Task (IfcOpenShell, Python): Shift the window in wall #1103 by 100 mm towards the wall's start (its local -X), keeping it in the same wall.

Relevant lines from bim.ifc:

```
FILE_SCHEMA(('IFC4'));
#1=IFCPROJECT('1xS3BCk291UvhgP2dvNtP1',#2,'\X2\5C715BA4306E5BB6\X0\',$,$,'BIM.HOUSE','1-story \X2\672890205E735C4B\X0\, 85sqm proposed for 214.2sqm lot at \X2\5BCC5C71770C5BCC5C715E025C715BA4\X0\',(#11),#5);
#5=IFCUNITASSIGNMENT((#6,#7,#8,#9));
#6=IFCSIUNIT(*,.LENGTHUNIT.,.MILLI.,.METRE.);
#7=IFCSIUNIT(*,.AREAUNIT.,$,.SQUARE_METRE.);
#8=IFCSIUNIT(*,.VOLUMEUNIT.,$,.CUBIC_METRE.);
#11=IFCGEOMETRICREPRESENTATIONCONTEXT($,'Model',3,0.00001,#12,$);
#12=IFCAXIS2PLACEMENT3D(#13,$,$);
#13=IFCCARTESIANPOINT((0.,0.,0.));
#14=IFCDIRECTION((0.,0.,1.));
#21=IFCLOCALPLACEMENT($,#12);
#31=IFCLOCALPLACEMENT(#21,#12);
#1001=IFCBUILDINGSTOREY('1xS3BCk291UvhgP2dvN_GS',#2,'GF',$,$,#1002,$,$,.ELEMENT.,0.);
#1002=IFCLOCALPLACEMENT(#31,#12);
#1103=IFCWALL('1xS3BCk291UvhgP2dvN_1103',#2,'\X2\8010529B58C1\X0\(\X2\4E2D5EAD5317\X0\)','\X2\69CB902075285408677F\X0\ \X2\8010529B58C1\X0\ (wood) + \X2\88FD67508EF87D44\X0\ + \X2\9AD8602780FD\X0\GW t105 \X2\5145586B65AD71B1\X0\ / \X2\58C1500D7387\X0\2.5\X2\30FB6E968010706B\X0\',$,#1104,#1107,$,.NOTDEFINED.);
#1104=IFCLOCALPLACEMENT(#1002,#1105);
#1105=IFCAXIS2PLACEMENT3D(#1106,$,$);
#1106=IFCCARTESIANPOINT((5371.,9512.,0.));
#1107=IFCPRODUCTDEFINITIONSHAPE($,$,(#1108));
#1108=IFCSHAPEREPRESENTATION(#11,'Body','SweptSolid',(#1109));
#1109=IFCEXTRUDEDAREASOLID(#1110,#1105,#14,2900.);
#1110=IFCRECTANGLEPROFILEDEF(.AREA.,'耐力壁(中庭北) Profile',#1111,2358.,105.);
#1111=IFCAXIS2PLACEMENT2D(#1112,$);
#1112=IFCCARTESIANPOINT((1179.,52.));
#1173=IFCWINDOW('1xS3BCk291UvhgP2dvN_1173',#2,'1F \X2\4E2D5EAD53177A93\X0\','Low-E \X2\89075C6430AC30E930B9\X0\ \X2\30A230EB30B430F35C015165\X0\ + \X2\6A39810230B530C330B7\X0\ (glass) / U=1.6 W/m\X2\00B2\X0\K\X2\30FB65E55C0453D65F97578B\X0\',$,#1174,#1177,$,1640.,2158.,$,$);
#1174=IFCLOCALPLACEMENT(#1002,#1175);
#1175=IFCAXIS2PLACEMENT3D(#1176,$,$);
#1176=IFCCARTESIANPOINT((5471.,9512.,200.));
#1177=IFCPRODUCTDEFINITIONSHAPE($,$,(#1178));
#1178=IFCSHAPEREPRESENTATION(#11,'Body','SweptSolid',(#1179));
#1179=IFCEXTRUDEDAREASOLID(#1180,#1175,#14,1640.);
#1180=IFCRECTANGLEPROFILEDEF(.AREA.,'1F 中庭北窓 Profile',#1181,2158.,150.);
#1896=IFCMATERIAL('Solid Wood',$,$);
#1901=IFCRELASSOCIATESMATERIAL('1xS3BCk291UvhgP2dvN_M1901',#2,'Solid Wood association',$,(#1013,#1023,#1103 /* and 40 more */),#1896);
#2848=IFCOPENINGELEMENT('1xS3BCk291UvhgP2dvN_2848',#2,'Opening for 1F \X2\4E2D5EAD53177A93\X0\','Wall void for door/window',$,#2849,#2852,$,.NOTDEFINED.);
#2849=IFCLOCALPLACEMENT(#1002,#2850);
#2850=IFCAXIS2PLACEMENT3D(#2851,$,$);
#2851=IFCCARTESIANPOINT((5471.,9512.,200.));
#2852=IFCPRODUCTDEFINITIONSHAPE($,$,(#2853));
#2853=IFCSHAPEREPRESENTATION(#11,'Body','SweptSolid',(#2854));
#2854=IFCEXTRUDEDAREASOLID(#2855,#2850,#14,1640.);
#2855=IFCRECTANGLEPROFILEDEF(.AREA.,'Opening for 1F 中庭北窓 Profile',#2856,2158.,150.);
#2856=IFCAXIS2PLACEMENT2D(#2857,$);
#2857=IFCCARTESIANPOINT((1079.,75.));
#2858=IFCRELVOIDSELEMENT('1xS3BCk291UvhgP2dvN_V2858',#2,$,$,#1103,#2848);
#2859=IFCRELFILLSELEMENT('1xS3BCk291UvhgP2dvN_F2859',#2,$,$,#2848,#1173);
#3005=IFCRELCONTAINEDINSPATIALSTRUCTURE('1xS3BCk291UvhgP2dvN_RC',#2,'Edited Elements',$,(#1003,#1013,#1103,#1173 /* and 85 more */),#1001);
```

```python
import ifcopenshell
import ifcopenshell.api.geometry
import ifcopenshell.util.placement
import ifcopenshell.util.unit

model = ifcopenshell.open("bim.ifc")
unit_scale = ifcopenshell.util.unit.calculate_unit_scale(model)

window = model.by_id(1173)
opening = window.FillsVoids[0].RelatingOpeningElement
wall = opening.VoidsElements[0].RelatingBuildingElement

wall_matrix = ifcopenshell.util.placement.get_local_placement(wall.ObjectPlacement)
shift = wall_matrix[:3, 0] * -0.1 / unit_scale
before = ifcopenshell.util.placement.get_local_placement(window.ObjectPlacement)[:3, 3].copy()

# The window is not placed relative to its opening, so move both.
for product in (opening, window):
    matrix = ifcopenshell.util.placement.get_local_placement(product.ObjectPlacement)
    matrix[:3, 3] += shift
    ifcopenshell.api.geometry.edit_object_placement(model, product=product, matrix=matrix, is_si=False)

after = ifcopenshell.util.placement.get_local_placement(window.ObjectPlacement)[:3, 3]
print("window moved by", (after - before).round(3) + 0.0)

model.write("bim_updated.ifc")
```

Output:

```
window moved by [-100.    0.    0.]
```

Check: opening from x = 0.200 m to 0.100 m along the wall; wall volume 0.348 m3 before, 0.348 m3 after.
